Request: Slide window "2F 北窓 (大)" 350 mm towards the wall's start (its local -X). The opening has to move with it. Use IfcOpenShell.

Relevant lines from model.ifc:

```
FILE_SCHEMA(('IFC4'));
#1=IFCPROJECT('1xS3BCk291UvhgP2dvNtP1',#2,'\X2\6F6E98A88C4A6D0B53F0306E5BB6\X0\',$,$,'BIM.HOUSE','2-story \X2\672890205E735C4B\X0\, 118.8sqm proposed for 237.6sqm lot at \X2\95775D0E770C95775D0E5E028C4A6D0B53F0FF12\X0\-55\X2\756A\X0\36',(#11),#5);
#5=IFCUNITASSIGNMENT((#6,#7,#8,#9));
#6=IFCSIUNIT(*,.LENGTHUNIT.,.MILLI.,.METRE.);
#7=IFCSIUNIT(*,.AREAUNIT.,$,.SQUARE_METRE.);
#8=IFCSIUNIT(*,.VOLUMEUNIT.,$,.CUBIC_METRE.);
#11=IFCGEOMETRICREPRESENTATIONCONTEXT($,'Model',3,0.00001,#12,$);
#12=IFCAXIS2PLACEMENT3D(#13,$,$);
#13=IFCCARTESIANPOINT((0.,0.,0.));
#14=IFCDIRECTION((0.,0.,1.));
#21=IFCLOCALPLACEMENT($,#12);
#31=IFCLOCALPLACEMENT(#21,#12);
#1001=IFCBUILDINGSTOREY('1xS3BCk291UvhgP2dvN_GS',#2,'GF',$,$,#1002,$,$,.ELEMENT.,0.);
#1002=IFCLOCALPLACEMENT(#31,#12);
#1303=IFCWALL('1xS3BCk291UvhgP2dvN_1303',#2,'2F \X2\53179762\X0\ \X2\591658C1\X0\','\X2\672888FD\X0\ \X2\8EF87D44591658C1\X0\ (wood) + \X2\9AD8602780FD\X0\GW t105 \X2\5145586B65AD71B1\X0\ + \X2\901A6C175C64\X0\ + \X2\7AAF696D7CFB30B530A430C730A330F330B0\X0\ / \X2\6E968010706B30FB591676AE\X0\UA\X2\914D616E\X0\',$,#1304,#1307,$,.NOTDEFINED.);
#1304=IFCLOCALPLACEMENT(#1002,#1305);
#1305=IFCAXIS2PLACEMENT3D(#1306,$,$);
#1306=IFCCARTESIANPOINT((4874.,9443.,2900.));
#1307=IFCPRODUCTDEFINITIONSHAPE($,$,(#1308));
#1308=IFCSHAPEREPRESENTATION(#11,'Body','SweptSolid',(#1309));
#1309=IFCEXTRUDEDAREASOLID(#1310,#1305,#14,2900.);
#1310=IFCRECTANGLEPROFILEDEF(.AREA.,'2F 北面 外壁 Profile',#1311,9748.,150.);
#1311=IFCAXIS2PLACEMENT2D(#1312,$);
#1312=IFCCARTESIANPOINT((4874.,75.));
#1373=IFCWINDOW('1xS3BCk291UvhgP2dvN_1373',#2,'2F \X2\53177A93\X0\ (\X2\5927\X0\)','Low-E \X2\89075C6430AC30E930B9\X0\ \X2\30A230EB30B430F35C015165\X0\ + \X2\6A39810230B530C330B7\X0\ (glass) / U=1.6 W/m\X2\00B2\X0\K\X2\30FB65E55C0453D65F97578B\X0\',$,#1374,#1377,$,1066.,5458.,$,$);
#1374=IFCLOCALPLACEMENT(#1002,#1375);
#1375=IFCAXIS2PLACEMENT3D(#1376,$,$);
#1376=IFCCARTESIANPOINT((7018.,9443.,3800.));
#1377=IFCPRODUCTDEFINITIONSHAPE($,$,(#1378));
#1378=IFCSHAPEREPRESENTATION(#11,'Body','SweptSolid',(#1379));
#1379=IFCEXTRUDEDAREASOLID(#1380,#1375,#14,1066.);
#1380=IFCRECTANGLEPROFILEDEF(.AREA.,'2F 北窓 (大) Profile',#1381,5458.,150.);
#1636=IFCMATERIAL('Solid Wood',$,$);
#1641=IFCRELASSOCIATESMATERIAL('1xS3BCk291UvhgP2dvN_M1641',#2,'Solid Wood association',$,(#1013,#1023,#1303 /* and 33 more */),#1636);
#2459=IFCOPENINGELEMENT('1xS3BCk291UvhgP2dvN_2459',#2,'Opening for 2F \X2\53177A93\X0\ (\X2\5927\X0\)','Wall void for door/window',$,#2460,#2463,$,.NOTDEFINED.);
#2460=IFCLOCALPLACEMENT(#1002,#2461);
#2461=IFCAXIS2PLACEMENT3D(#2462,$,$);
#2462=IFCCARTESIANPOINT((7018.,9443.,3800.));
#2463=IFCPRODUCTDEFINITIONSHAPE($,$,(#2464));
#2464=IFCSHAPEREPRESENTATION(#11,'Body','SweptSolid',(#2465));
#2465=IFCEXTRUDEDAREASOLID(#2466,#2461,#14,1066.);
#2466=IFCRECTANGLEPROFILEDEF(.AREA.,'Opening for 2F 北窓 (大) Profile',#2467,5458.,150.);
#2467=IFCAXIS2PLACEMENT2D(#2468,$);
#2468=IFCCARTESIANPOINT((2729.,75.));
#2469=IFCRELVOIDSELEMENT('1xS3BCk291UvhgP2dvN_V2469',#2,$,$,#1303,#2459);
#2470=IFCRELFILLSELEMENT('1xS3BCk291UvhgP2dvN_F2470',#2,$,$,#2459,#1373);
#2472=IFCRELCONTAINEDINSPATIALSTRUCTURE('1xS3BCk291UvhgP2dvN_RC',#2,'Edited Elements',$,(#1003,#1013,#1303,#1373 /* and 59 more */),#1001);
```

```python
import ifcopenshell
import ifcopenshell.api.geometry
import ifcopenshell.util.placement

model = ifcopenshell.open("model.ifc")

window = model.by_guid("1xS3BCk291UvhgP2dvN_1373")
opening = window.FillsVoids[0].RelatingOpeningElement
wall = opening.VoidsElements[0].RelatingBuildingElement

wall_matrix = ifcopenshell.util.placement.get_local_placement(wall.ObjectPlacement)
shift = wall_matrix[:3, 0] * -350.0
before = ifcopenshell.util.placement.get_local_placement(window.ObjectPlacement)[:3, 3].copy()

# The window is not placed relative to its opening, so move both.
for product in (opening, window):
    matrix = ifcopenshell.util.placement.get_local_placement(product.ObjectPlacement)
    matrix[:3, 3] += shift
    ifcopenshell.api.geometry.edit_object_placement(model, product=product, matrix=matrix, is_si=False)

after = ifcopenshell.util.placement.get_local_placement(window.ObjectPlacement)[:3, 3]
print("window moved by", (after - before).round(3) + 0.0)

model.write("model_updated.ifc")
```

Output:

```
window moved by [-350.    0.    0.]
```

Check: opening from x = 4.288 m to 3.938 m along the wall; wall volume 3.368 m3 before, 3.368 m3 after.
